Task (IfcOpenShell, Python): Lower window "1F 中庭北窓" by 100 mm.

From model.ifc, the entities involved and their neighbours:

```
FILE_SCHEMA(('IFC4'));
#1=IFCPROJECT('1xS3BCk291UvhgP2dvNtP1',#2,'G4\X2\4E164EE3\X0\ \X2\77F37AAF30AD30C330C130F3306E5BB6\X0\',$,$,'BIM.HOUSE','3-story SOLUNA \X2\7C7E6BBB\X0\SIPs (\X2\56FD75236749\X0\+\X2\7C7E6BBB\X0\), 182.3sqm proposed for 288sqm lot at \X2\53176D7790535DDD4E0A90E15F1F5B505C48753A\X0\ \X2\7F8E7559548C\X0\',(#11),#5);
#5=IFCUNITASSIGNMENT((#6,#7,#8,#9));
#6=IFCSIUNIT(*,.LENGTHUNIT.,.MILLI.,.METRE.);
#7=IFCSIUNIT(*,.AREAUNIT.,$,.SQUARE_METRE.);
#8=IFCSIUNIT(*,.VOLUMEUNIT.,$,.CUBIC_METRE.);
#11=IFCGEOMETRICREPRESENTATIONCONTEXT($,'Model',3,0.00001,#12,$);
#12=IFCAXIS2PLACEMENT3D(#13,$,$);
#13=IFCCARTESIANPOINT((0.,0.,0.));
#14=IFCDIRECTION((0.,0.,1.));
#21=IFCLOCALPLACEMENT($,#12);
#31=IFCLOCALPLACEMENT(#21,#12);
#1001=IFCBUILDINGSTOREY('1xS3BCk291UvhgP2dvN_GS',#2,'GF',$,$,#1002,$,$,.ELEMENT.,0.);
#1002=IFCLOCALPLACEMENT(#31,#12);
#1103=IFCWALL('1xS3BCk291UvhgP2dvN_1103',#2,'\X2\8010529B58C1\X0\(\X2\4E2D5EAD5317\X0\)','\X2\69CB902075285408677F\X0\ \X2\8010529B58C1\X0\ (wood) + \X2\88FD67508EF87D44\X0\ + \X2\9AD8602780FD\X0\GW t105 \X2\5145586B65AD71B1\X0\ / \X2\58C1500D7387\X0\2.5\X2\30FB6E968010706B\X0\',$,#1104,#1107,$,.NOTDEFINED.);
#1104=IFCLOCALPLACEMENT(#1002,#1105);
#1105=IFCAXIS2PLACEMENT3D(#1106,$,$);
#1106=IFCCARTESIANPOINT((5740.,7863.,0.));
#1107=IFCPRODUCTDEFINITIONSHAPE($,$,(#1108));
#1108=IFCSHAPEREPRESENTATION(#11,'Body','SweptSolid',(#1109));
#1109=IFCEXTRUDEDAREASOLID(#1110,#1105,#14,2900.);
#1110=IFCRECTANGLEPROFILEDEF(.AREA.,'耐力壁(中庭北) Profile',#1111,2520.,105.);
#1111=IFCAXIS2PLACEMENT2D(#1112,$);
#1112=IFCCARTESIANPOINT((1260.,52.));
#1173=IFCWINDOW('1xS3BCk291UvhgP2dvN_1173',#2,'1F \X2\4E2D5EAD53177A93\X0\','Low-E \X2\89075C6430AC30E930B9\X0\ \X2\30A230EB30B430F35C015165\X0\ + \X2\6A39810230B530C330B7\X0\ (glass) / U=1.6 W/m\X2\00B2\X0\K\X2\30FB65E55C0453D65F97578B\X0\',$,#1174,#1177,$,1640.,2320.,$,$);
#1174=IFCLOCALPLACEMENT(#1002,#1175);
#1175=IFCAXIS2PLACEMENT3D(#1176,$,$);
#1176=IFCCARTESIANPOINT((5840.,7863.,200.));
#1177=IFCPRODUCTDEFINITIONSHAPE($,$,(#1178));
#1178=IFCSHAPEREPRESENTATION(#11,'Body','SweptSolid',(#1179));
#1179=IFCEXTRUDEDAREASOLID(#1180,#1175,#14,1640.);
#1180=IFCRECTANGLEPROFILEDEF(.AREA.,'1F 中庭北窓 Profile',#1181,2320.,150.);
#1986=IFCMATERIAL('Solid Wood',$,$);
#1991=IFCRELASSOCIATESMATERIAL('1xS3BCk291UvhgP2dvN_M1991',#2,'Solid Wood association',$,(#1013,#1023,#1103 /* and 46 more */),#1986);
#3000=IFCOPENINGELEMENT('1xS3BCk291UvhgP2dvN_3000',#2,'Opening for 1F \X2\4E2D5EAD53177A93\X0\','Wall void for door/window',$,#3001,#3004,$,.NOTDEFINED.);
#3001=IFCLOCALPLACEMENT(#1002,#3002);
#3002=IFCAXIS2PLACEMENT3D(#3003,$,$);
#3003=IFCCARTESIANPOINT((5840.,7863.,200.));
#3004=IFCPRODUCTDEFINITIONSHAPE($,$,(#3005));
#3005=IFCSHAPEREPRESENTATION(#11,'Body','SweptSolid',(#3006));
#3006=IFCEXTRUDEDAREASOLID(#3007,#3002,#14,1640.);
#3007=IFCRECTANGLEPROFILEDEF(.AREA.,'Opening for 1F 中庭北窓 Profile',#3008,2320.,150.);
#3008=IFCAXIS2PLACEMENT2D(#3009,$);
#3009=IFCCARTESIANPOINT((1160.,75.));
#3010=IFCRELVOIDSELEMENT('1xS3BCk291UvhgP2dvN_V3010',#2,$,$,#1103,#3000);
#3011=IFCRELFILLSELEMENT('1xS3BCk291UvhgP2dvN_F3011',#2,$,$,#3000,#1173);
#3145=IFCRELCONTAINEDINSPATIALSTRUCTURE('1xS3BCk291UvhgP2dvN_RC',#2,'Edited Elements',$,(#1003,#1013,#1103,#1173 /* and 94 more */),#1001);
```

```python
import numpy as np
import ifcopenshell
import ifcopenshell.api.geometry
import ifcopenshell.util.placement
import ifcopenshell.util.unit

model = ifcopenshell.open("model.ifc")
unit_scale = ifcopenshell.util.unit.calculate_unit_scale(model)

window = model.by_guid("1xS3BCk291UvhgP2dvN_1173")
opening = window.FillsVoids[0].RelatingOpeningElement
dz = -0.1 / unit_scale

shift = np.array([0.0, 0.0, dz])
# The window is not placed relative to its opening, so move both.
for product in (opening, window):
    matrix = ifcopenshell.util.placement.get_local_placement(product.ObjectPlacement)
    matrix[:3, 3] += shift
    ifcopenshell.api.geometry.edit_object_placement(model, product=product, matrix=matrix, is_si=False)

print(f"moved by {dz * unit_scale:+.3f} m")

model.write("model_v2.ifc")
```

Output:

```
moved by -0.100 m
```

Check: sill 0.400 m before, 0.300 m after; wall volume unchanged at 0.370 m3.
